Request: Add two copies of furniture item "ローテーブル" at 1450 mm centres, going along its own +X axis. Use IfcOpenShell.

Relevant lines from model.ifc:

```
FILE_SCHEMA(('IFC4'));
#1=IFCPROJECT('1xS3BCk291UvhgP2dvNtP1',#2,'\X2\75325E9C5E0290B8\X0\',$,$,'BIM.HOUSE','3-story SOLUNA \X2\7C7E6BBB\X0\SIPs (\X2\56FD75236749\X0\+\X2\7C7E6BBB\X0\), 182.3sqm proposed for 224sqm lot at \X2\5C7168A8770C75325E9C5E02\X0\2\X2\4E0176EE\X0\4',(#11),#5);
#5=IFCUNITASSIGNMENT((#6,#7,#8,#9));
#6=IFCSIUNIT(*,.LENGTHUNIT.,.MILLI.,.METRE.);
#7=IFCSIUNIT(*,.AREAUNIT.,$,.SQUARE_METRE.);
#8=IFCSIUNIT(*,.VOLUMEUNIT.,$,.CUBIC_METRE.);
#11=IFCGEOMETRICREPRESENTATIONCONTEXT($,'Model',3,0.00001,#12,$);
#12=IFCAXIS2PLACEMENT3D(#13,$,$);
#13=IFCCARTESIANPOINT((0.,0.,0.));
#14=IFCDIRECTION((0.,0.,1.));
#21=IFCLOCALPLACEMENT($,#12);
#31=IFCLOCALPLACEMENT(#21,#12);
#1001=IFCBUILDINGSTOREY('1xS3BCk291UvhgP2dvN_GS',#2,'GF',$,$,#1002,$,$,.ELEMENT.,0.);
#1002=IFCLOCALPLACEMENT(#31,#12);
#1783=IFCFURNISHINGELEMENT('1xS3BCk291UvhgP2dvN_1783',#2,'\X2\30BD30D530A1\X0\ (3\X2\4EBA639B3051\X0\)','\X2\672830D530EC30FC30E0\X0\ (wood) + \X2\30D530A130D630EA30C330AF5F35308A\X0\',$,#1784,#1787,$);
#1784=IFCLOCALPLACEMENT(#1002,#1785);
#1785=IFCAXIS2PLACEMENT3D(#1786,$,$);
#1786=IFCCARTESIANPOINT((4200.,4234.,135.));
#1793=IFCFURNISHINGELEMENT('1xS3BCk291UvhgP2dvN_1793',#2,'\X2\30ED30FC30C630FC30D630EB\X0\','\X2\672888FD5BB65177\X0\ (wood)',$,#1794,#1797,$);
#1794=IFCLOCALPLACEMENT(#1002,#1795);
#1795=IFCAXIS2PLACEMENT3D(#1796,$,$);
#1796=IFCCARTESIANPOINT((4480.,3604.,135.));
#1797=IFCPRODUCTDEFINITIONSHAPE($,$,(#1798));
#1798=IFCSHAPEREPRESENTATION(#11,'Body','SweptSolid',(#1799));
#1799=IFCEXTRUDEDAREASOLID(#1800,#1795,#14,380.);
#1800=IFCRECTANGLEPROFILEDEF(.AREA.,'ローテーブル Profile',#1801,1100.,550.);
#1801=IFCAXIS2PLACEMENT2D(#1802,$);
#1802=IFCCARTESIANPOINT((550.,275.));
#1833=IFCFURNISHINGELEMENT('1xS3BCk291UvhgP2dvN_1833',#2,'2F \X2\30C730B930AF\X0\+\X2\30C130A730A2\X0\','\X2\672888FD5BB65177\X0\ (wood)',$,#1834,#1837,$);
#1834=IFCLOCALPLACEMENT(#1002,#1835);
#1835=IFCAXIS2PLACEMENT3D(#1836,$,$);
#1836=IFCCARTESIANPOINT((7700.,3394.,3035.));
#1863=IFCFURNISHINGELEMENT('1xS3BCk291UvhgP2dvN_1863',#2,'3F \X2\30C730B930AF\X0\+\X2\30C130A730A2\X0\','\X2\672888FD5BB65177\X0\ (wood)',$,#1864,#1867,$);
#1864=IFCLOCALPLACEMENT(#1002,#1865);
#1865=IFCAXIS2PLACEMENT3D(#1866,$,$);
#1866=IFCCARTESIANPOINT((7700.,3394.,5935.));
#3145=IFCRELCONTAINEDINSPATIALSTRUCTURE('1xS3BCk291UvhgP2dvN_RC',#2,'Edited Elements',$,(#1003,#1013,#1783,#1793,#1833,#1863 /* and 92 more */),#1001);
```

```python
import ifcopenshell
import ifcopenshell.api.geometry
import ifcopenshell.api.root
import ifcopenshell.util.element
import ifcopenshell.util.placement

model = ifcopenshell.open("model.ifc")


def reuse_history(source, copy):
    """copy_class also copies each property set's owner history, people and application; keep the originals."""
    for rel in copy.IsDefinedBy:
        if rel.is_a("IfcRelDefinesByProperties") and (history := rel.RelatingPropertyDefinition.OwnerHistory):
            rel.RelatingPropertyDefinition.OwnerHistory = source.OwnerHistory
            ifcopenshell.util.element.remove_deep2(model, history)


source = model.by_guid("1xS3BCk291UvhgP2dvN_1793")
base = ifcopenshell.util.placement.get_local_placement(source.ObjectPlacement)
step = base[:3, 0] * 1450.0

for i in range(1, 3):
    copy = ifcopenshell.api.root.copy_class(model, product=source)
    copy.Representation = ifcopenshell.util.element.copy_deep(
        model, source.Representation, exclude=["IfcGeometricRepresentationContext", "IfcRepresentationMap"]
    )
    reuse_history(source, copy)
    matrix = base.copy()
    matrix[:3, 3] += i * step
    print("added at", matrix[:3, 3].round(3) + 0.0)
    ifcopenshell.api.geometry.edit_object_placement(model, product=copy, matrix=matrix, is_si=False)

model.write("model_v2.ifc")
```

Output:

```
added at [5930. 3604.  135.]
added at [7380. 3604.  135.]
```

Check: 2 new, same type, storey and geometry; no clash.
